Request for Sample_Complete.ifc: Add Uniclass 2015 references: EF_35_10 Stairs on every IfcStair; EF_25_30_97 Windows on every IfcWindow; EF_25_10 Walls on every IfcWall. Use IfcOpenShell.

First a look at what the model holds.

```python
import ifcopenshell

model = ifcopenshell.open("Sample_Complete.ifc")
print(model.schema)
print("classifications:", [c.Name for c in model.by_type("IfcClassification")])
for ifc_class in ("IfcDoor", "IfcRoof", "IfcStair", "IfcWall", "IfcWindow"):
    print(ifc_class, len(model.by_type(ifc_class)))
```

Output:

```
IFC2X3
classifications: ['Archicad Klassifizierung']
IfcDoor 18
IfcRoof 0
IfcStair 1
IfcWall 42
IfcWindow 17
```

```python
import ifcopenshell
import ifcopenshell.api.classification

model = ifcopenshell.open("Sample_Complete.ifc")

# IFC2X3 requires Source and Edition and has no link from the project to the system.
system = model.create_entity("IfcClassification", Source="NBS", Edition="2015", Name="Uniclass 2015")

codes = {
    "IfcStair": ("EF_35_10", "Stairs"),
    "IfcWindow": ("EF_25_30_97", "Windows"),
    "IfcWall": ("EF_25_10", "Walls"),
}
for ifc_class, (code, name) in codes.items():
    products = model.by_type(ifc_class)
    ifcopenshell.api.classification.add_reference(
        model, products=products, classification=system, identification=code, name=name
    )
    print(code, len(products))

model.write("Sample_Complete_v2.ifc")
```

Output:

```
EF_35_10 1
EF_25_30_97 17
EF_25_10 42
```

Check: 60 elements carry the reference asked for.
